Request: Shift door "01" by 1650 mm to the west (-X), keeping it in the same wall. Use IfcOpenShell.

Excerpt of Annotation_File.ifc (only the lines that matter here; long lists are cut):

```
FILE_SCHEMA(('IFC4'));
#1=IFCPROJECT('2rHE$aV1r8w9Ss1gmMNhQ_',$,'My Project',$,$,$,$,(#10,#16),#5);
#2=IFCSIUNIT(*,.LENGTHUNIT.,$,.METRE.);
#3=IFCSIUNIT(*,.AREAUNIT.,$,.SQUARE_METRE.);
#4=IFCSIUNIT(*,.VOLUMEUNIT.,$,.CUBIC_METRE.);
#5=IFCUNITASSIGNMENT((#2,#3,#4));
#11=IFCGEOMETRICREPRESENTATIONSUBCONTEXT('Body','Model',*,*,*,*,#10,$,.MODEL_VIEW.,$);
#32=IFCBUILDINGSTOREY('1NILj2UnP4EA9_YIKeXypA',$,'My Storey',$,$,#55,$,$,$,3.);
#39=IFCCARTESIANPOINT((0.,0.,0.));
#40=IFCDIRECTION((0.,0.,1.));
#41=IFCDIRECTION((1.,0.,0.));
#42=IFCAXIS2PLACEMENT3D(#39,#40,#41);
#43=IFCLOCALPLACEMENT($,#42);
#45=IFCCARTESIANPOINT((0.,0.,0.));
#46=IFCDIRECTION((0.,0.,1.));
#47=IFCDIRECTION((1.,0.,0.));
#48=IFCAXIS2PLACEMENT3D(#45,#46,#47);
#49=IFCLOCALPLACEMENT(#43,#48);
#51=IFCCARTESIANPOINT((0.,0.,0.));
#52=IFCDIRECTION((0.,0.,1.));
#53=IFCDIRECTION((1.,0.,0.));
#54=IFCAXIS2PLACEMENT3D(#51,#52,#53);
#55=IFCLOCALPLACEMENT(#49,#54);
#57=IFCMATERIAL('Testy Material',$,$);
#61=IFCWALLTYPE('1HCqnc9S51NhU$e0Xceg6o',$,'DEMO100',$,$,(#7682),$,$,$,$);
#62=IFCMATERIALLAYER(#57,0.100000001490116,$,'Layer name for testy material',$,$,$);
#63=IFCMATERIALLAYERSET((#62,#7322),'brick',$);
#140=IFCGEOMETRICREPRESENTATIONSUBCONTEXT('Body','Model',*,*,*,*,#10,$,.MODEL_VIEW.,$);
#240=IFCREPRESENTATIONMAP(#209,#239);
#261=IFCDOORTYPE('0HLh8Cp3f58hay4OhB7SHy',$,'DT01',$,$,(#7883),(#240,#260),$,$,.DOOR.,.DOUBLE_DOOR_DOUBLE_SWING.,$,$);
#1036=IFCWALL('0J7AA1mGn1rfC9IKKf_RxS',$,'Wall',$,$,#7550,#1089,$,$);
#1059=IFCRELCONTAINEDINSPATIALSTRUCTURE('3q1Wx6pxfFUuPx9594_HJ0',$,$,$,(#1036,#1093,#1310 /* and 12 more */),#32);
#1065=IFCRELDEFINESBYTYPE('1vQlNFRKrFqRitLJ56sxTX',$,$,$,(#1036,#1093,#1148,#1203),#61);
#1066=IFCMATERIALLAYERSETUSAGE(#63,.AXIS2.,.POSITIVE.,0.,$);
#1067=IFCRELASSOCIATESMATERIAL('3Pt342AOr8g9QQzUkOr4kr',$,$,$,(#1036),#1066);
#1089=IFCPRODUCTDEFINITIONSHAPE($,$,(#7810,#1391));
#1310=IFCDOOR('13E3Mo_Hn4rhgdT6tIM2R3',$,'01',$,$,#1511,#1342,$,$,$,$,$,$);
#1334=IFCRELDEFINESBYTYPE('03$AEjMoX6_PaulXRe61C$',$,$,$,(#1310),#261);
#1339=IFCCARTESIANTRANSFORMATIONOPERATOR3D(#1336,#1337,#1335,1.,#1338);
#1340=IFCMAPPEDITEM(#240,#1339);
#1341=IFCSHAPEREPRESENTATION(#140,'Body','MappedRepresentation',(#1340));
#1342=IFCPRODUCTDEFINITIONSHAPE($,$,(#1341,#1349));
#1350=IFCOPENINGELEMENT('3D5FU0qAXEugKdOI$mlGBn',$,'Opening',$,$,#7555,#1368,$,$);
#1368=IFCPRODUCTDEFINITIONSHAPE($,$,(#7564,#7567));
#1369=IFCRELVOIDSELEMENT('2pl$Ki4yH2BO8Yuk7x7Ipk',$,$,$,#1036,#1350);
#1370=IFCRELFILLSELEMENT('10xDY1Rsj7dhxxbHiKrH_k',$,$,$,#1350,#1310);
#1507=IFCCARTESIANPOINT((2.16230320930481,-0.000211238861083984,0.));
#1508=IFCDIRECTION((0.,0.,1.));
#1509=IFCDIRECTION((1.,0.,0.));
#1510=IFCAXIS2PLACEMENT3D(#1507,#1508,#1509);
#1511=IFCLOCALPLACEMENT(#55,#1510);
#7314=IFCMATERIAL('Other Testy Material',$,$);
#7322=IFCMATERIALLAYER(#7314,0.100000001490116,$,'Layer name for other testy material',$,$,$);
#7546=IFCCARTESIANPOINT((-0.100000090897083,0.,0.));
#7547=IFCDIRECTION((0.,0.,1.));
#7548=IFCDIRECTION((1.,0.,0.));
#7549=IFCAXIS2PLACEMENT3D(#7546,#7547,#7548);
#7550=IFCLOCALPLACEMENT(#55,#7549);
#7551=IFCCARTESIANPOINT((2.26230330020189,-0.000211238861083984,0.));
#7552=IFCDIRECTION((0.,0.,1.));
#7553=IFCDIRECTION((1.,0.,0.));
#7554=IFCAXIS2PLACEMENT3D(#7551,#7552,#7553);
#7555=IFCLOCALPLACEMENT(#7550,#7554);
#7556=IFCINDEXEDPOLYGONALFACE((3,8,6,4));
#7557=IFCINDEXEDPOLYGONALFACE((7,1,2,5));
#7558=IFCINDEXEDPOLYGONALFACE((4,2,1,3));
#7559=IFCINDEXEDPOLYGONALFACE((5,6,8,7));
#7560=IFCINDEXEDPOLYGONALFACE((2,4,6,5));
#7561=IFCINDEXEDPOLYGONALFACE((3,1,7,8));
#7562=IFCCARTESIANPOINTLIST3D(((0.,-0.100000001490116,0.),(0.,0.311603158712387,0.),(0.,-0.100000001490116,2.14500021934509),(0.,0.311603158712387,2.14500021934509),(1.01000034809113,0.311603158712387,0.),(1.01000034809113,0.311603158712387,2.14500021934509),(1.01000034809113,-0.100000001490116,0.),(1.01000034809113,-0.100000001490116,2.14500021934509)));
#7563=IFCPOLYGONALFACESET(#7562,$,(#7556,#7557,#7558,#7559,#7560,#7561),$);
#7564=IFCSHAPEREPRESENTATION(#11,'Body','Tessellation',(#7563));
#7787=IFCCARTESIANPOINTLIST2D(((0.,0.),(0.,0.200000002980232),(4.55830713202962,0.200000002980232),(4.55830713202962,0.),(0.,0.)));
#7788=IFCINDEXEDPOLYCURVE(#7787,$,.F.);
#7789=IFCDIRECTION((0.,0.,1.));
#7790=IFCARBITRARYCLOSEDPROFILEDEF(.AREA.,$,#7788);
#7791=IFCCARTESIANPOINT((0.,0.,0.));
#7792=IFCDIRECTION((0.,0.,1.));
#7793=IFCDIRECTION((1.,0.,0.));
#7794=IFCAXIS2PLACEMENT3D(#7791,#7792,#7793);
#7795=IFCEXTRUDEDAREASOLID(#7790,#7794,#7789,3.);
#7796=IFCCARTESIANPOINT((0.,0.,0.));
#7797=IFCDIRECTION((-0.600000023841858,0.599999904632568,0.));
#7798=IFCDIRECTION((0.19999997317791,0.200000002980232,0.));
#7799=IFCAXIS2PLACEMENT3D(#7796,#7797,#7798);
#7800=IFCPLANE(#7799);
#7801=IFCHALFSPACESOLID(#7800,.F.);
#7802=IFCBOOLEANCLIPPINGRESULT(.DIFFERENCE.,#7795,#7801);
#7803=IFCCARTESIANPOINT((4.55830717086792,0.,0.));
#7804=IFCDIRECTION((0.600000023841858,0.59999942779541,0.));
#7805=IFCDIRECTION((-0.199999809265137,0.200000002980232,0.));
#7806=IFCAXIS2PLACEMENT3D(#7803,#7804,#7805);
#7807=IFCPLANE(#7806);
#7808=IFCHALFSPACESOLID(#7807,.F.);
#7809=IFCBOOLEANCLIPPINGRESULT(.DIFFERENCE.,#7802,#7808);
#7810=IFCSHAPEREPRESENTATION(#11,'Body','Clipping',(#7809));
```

```python
import ifcopenshell
import ifcopenshell.api.geometry
import ifcopenshell.util.placement

model = ifcopenshell.open("Annotation_File.ifc")

door = model.by_guid("13E3Mo_Hn4rhgdT6tIM2R3")
opening = door.FillsVoids[0].RelatingOpeningElement
wall = opening.VoidsElements[0].RelatingBuildingElement

wall_matrix = ifcopenshell.util.placement.get_local_placement(wall.ObjectPlacement)
shift = wall_matrix[:3, 0] * -1.65
before = ifcopenshell.util.placement.get_local_placement(door.ObjectPlacement)[:3, 3].copy()

# The door is not placed relative to its opening, so move both.
for product in (opening, door):
    matrix = ifcopenshell.util.placement.get_local_placement(product.ObjectPlacement)
    matrix[:3, 3] += shift
    ifcopenshell.api.geometry.edit_object_placement(model, product=product, matrix=matrix, is_si=False)

after = ifcopenshell.util.placement.get_local_placement(door.ObjectPlacement)[:3, 3]
print("door moved by", (after - before).round(3) + 0.0)

model.write("Annotation_File-out.ifc")
```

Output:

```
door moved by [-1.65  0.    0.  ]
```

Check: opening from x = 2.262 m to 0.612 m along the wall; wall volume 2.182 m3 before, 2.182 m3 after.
